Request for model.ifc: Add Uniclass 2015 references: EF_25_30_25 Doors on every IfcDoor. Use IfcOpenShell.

First a look at what the model holds.

```python
import ifcopenshell

model = ifcopenshell.open("model.ifc")
print(model.schema)
print("classifications:", [c.Name for c in model.by_type("IfcClassification")])
for ifc_class in ("IfcDoor", "IfcRoof", "IfcStair", "IfcWall", "IfcWindow"):
    print(ifc_class, len(model.by_type(ifc_class)))
```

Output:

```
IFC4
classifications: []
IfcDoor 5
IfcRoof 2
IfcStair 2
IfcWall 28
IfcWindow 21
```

```python
import ifcopenshell
import ifcopenshell.api.classification

model = ifcopenshell.open("model.ifc")

system = ifcopenshell.api.classification.add_classification(model, classification="Uniclass 2015")

codes = {
    "IfcDoor": ("EF_25_30_25", "Doors"),
}
for ifc_class, (code, name) in codes.items():
    products = model.by_type(ifc_class)
    ifcopenshell.api.classification.add_reference(
        model, products=products, classification=system, identification=code, name=name
    )
    print(code, len(products))

model.write("model_rev.ifc")
```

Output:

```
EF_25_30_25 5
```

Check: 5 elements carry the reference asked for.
